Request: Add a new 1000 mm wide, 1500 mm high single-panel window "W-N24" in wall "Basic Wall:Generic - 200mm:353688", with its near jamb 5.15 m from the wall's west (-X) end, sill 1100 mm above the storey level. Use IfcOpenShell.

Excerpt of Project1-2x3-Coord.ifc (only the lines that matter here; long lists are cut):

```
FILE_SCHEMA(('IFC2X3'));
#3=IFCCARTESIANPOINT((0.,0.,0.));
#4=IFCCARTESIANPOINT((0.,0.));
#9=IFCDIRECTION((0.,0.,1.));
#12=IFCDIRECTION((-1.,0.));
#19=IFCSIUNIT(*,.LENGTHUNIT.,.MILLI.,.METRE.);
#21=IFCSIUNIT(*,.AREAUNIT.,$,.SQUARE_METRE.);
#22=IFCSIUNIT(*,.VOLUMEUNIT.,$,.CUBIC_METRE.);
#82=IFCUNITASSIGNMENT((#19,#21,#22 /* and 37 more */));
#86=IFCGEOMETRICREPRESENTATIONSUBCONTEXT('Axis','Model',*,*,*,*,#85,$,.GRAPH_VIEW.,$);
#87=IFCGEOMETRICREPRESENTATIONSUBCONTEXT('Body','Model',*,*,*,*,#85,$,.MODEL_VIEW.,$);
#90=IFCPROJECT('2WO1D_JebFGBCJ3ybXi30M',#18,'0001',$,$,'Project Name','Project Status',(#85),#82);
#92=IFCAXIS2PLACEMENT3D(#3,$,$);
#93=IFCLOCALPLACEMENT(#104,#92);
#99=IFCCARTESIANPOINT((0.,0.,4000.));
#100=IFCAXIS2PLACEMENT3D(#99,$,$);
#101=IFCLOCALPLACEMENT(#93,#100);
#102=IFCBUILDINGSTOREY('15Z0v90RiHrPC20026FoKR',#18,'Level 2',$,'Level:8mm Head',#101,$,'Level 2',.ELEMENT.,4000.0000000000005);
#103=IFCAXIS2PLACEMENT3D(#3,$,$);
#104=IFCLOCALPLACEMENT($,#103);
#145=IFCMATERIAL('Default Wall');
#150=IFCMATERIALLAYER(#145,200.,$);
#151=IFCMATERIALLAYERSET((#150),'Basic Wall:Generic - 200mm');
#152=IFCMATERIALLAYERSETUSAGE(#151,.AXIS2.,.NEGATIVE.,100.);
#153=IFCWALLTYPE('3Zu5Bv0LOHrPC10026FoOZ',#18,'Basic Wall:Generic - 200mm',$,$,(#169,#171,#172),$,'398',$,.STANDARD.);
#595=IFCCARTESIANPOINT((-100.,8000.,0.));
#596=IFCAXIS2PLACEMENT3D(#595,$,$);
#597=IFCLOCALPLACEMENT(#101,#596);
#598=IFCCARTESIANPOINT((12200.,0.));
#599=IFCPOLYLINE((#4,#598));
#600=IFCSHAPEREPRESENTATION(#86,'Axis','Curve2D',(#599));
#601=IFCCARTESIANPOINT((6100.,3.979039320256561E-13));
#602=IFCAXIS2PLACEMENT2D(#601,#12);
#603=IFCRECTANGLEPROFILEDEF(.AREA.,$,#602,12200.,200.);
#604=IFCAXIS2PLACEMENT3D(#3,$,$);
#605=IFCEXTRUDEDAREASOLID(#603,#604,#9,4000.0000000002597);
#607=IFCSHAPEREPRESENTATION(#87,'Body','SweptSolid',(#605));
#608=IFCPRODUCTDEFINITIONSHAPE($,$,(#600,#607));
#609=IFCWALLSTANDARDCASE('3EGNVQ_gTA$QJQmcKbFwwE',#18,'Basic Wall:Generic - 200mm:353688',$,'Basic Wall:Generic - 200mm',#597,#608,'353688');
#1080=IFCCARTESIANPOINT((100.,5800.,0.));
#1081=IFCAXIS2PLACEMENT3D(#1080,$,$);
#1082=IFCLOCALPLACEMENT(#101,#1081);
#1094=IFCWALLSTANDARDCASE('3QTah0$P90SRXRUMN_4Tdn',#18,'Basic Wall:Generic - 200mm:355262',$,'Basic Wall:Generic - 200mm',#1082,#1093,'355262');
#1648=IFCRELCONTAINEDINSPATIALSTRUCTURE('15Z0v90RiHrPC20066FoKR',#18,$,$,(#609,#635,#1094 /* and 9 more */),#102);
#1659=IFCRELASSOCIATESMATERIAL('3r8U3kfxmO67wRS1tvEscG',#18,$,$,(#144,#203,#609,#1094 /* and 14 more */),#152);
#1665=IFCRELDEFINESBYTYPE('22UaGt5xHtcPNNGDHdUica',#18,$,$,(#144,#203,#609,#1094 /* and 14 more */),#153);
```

```python
import numpy as np
import ifcopenshell
import ifcopenshell.api.feature
import ifcopenshell.api.geometry
import ifcopenshell.api.root
import ifcopenshell.api.spatial
import ifcopenshell.api.type
import ifcopenshell.geom
import ifcopenshell.util.element
import ifcopenshell.util.placement
import ifcopenshell.util.representation
import ifcopenshell.util.shape
import ifcopenshell.util.unit

model = ifcopenshell.open("Project1-2x3-Coord.ifc")
unit_scale = ifcopenshell.util.unit.calculate_unit_scale(model)
settings = ifcopenshell.geom.settings()


def volume(element):
    """Net volume in cubic metres, openings subtracted."""
    shape = ifcopenshell.geom.create_shape(settings, element)
    return ifcopenshell.util.shape.get_volume(shape.geometry)


wall = model.by_id(609)
storey = ifcopenshell.util.element.get_container(wall, ifc_class="IfcBuildingStorey")
context = ifcopenshell.util.representation.get_context(model, "Model", "Body", "MODEL_VIEW")
before = volume(wall)

width, height, from_end, sill = 1, 1.5, 5.15, 1.1  # metres

# The wall runs along its own X axis, and the end named is its -X end.
wall_shape = ifcopenshell.geom.create_shape(settings, wall)
x, y, z = ifcopenshell.util.shape.get_vertices(wall_shape.geometry).T
start = x.min() + from_end
face, thickness = float(y.min()), float(y.max() - y.min())
wall_matrix = ifcopenshell.util.placement.get_local_placement(wall.ObjectPlacement)
level = ifcopenshell.util.placement.get_local_placement(storey.ObjectPlacement)[2, 3]


def in_wall(x, y):
    """Placement at x, y metres in the wall's axes, at sill height."""
    matrix = wall_matrix.copy()
    matrix[:, 3] = wall_matrix @ np.array([x / unit_scale, y / unit_scale, 0.0, 1.0])
    matrix[2, 3] = level + sill / unit_scale
    return matrix


# Opening: a box that overshoots both wall faces by 50 mm.
opening = ifcopenshell.api.root.create_entity(model, ifc_class="IfcOpeningElement")
box = ifcopenshell.api.geometry.add_wall_representation(
    model, context=context, length=width, height=height, thickness=thickness + 0.1
)
ifcopenshell.api.geometry.assign_representation(model, product=opening, representation=box)
ifcopenshell.api.geometry.edit_object_placement(model, product=opening, matrix=in_wall(start, face - 0.05), is_si=False)
ifcopenshell.api.feature.add_feature(model, feature=opening, element=wall)

window = ifcopenshell.api.root.create_entity(model, ifc_class="IfcWindow", name="W-N24")
window.OverallWidth, window.OverallHeight = width / unit_scale, height / unit_scale
body = ifcopenshell.api.geometry.add_window_representation(
    model,
    context=context,
    overall_width=window.OverallWidth,
    overall_height=window.OverallHeight,
    partition_type="SINGLE_PANEL",
)
ifcopenshell.api.geometry.assign_representation(model, product=window, representation=body)
ifcopenshell.api.spatial.assign_container(model, products=[window], relating_structure=storey)
fills = ifcopenshell.api.feature.add_filling(model, opening=opening, element=window)
fills.OwnerHistory = window.OwnerHistory  # required in IFC2X3

# IFC2X3 keeps the operation on the window style.
style = ifcopenshell.api.root.create_entity(model, ifc_class="IfcWindowStyle", name="W-N24")
style.OperationType, style.ConstructionType = "SINGLE_PANEL", "NOTDEFINED"
style.ParameterTakesPrecedence = style.Sizeable = False
ifcopenshell.api.type.assign_type(model, related_objects=[window], relating_type=style)

# Centre the window in the wall's thickness.
ifcopenshell.api.geometry.edit_object_placement(model, product=window, matrix=in_wall(start, face), is_si=False)
window_shape = ifcopenshell.geom.create_shape(settings, window)
depth = ifcopenshell.util.shape.get_vertices(window_shape.geometry)[:, 1]
offset = face + thickness / 2 - (depth.min() + depth.max()) / 2
ifcopenshell.api.geometry.edit_object_placement(model, product=window, matrix=in_wall(start, offset), is_si=False)

after = volume(wall)

print(f"wall volume {before:.3f} -> {after:.3f} m3")

model.write("Project1-2x3-Coord-out.ifc")
```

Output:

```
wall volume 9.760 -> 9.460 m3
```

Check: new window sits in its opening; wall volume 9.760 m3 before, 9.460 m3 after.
